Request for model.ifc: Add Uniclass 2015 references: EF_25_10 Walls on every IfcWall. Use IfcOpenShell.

First a look at what the model holds.

```python
import ifcopenshell

model = ifcopenshell.open("model.ifc")
print(model.schema)
print("classifications:", [c.Name for c in model.by_type("IfcClassification")])
for ifc_class in ("IfcDoor", "IfcRoof", "IfcStair", "IfcWall", "IfcWindow"):
    print(ifc_class, len(model.by_type(ifc_class)))
```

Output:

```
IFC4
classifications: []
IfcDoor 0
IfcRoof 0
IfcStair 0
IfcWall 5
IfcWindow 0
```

```python
import ifcopenshell
import ifcopenshell.api.classification

model = ifcopenshell.open("model.ifc")

system = ifcopenshell.api.classification.add_classification(model, classification="Uniclass 2015")

codes = {
    "IfcWall": ("EF_25_10", "Walls"),
}
for ifc_class, (code, name) in codes.items():
    products = model.by_type(ifc_class)
    ifcopenshell.api.classification.add_reference(
        model, products=products, classification=system, identification=code, name=name
    )
    print(code, len(products))

model.write("model-out.ifc")
```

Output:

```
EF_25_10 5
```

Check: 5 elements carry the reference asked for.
